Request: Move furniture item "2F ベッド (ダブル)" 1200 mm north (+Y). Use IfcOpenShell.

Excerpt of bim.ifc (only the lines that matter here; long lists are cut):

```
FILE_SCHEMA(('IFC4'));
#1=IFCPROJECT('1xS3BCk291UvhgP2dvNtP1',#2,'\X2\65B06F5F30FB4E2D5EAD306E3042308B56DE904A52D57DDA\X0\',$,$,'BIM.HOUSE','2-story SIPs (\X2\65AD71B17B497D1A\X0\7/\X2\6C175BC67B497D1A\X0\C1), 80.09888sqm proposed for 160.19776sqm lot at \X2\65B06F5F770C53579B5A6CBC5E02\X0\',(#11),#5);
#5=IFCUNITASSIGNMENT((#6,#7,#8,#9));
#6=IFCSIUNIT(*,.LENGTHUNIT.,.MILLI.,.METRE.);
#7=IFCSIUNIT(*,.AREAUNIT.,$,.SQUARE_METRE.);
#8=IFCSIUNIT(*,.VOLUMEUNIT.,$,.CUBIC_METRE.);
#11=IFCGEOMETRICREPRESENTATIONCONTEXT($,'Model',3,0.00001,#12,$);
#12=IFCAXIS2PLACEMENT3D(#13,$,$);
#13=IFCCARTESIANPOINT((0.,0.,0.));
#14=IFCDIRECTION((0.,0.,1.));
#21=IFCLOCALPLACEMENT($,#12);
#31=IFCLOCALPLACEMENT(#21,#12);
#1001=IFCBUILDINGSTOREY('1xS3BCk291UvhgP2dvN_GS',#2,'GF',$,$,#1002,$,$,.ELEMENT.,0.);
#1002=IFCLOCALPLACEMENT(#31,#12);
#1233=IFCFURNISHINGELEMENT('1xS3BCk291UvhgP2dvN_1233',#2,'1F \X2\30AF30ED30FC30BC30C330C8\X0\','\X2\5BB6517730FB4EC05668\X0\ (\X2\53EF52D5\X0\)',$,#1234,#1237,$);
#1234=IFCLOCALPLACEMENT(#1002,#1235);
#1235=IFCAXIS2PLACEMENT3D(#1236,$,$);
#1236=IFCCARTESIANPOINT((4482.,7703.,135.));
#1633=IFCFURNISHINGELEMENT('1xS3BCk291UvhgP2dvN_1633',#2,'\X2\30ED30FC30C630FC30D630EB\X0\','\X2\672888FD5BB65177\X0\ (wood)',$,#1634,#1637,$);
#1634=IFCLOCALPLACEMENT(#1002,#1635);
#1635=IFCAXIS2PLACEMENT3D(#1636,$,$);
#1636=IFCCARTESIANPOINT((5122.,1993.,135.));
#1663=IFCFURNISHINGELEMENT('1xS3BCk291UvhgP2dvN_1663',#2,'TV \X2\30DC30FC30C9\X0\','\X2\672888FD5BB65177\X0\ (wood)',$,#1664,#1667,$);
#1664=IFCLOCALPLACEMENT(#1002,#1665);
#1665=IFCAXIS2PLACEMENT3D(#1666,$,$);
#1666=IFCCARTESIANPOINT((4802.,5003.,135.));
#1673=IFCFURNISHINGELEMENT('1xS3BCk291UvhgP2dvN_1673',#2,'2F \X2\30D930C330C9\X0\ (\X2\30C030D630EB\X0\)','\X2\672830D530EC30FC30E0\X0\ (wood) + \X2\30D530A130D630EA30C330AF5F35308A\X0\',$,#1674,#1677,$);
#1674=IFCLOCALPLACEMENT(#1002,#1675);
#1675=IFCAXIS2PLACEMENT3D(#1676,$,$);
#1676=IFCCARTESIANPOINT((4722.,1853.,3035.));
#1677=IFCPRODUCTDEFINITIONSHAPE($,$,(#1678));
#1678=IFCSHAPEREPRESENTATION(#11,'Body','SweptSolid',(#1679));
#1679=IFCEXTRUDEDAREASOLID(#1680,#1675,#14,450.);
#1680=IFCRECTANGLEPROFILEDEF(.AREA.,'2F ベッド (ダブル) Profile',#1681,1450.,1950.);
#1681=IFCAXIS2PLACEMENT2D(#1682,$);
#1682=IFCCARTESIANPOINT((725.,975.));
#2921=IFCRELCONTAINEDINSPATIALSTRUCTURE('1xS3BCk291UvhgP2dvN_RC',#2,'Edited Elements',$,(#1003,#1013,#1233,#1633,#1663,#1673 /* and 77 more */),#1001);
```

```python
import ifcopenshell
import ifcopenshell.api.geometry
import ifcopenshell.util.placement

model = ifcopenshell.open("bim.ifc")

item = model.by_guid("1xS3BCk291UvhgP2dvN_1673")
matrix = ifcopenshell.util.placement.get_local_placement(item.ObjectPlacement)
matrix[1, 3] += 1200.0
ifcopenshell.api.geometry.edit_object_placement(model, product=item, matrix=matrix, is_si=False)

print(ifcopenshell.util.placement.get_local_placement(item.ObjectPlacement).round(3) + 0.0)

model.write("bim_edited.ifc")
```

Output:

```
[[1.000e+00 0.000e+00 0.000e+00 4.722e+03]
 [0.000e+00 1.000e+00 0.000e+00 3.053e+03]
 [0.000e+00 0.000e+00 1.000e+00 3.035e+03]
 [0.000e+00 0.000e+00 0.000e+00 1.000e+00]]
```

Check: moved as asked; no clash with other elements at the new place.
